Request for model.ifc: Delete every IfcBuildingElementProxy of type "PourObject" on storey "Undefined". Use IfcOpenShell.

First a look at what the model holds.

```python
import ifcopenshell
import ifcopenshell.util.element

model = ifcopenshell.open("model.ifc")
print(model.schema)
storey = next(s for s in model.by_type("IfcBuildingStorey") if s.Name == "Undefined")
proxies = [e for e in ifcopenshell.util.element.get_decomposition(storey) if e.is_a("IfcBuildingElementProxy")]
seen = {}
for e in proxies:
    element_type = ifcopenshell.util.element.get_type(e)
    name = element_type.Name if element_type not in (None, e) else None
    seen[name] = seen.get(name, 0) + 1
for name, count in sorted(seen.items(), key=str):
    print(count, "x", name)
```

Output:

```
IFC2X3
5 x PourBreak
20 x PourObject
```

```python
import ifcopenshell
import ifcopenshell.api.root
import ifcopenshell.util.element

model = ifcopenshell.open("model.ifc")

storey = next(s for s in model.by_type("IfcBuildingStorey") if s.Name == "Undefined")
proxies = [e for e in ifcopenshell.util.element.get_decomposition(storey) if e.is_a("IfcBuildingElementProxy")]
targets = [e for e in proxies if (t := ifcopenshell.util.element.get_type(e)) not in (None, e) and t.Name == "PourObject"]

for e in targets:
    ifcopenshell.api.root.remove_product(model, product=e)
print(len(targets), "removed")

model.write("model_rev.ifc")
```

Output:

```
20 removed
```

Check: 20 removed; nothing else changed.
